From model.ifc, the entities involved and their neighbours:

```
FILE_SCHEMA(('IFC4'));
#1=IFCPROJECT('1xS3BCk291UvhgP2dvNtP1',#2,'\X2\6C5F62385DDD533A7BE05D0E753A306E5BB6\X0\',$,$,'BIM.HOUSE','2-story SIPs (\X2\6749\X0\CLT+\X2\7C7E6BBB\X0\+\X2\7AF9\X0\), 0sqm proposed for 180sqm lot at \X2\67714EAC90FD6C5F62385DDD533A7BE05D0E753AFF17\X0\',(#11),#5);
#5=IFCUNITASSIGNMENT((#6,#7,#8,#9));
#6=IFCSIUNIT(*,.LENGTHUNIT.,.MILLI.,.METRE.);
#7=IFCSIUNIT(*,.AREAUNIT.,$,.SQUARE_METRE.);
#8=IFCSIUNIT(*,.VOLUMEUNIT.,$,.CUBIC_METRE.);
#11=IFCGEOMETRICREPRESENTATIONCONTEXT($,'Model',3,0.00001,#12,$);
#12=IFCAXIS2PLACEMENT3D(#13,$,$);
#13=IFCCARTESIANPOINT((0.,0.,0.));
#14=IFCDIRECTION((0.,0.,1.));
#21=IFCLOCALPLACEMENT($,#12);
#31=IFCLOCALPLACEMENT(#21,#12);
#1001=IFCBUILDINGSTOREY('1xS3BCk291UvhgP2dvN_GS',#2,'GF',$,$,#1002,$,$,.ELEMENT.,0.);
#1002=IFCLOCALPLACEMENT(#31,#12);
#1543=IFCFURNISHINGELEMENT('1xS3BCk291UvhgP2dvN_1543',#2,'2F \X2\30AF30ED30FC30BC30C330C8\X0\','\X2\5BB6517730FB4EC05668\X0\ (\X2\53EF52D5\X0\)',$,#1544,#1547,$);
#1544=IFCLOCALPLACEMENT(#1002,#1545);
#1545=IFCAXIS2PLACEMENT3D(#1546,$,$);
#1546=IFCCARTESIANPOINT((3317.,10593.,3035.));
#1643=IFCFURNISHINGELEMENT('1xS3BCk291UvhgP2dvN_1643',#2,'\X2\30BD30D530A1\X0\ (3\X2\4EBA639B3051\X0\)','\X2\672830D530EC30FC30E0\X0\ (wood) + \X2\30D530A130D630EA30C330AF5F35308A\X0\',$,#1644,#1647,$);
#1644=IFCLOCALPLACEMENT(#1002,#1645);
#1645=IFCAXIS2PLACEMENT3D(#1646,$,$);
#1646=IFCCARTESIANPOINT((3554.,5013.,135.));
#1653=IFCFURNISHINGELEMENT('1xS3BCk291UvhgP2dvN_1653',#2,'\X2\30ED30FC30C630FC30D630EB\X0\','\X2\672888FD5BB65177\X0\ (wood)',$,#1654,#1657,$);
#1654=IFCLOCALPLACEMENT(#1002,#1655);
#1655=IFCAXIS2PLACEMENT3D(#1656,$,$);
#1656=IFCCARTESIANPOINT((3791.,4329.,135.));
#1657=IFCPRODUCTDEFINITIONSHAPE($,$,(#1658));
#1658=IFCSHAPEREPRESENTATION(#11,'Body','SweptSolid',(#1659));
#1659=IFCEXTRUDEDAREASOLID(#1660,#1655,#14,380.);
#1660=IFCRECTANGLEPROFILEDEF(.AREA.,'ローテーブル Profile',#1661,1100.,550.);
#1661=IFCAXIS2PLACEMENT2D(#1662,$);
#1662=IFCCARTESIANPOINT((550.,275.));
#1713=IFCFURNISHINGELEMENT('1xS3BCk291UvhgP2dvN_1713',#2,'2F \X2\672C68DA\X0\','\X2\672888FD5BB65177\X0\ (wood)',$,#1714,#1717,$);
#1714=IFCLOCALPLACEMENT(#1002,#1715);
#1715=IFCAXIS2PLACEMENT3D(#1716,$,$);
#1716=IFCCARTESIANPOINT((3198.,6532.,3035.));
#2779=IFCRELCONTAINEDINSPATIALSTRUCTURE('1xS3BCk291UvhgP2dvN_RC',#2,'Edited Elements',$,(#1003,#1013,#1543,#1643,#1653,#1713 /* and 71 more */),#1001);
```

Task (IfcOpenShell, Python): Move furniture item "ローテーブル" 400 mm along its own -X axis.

```python
import ifcopenshell
import ifcopenshell.api.geometry
import ifcopenshell.util.placement

model = ifcopenshell.open("model.ifc")

item = model.by_id(1653)
matrix = ifcopenshell.util.placement.get_local_placement(item.ObjectPlacement)
matrix[:3, 3] -= matrix[:3, 0] * 400.0
ifcopenshell.api.geometry.edit_object_placement(model, product=item, matrix=matrix, is_si=False)

print(ifcopenshell.util.placement.get_local_placement(item.ObjectPlacement).round(3) + 0.0)

model.write("model_rev.ifc")
```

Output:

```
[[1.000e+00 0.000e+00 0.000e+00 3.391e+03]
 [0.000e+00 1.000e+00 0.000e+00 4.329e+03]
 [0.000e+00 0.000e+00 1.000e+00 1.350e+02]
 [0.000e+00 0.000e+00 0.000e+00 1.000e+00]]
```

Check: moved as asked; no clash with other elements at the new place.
